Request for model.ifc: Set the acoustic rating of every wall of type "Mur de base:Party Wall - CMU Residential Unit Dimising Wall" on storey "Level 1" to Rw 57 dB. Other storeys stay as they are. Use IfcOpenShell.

First a look at what the model holds.

```python
import ifcopenshell
import ifcopenshell.util.element

model = ifcopenshell.open("model.ifc")
print(model.schema)
storey = next(s for s in model.by_type("IfcBuildingStorey") if s.Name == "Level 1")
walls = [e for e in ifcopenshell.util.element.get_decomposition(storey) if e.is_a("IfcWall")]
seen = {}
for e in walls:
    element_type = ifcopenshell.util.element.get_type(e)
    key = (element_type.Name if element_type != e and element_type else None, ifcopenshell.util.element.get_pset(e, "Pset_WallCommon", "AcousticRating"))
    seen[key] = seen.get(key, 0) + 1
for (name, value), count in sorted(seen.items(), key=str):
    print(count, "x", name, "|", value)
```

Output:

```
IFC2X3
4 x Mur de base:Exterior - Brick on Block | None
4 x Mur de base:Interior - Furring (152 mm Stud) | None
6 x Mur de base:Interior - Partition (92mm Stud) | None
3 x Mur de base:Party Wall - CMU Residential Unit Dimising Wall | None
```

```python
import ifcopenshell
import ifcopenshell.api.pset
import ifcopenshell.util.element

model = ifcopenshell.open("model.ifc")

storey = next(s for s in model.by_type("IfcBuildingStorey") if s.Name == "Level 1")
walls = [e for e in ifcopenshell.util.element.get_decomposition(storey) if e.is_a("IfcWall")]

count = 0
for e in walls:
    element_type = ifcopenshell.util.element.get_type(e)
    if element_type in (None, e) or element_type.Name != "Mur de base:Party Wall - CMU Residential Unit Dimising Wall":
        continue
    # add_pset returns the element's existing set when there is one.
    pset = ifcopenshell.api.pset.add_pset(model, product=e, name="Pset_WallCommon")
    ifcopenshell.api.pset.edit_pset(model, pset=pset, properties={"AcousticRating": "Rw 57 dB"})
    count += 1

print(count, "walls updated")

model.write("model_rev.ifc")
```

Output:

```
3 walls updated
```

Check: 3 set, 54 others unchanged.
